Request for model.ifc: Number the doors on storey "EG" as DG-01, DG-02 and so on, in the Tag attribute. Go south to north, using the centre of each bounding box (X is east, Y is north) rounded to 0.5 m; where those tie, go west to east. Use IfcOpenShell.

First a look at what the model holds.

```python
import ifcopenshell
import ifcopenshell.util.element
import ifcopenshell.util.placement

model = ifcopenshell.open("model.ifc")
print(model.schema)
storey = next(s for s in model.by_type("IfcBuildingStorey") if s.Name == "EG")
doors = [e for e in ifcopenshell.util.element.get_decomposition(storey) if e.is_a("IfcDoor")]
for e in sorted(doors, key=lambda e: e.id()):
    origin = ifcopenshell.util.placement.get_local_placement(e.ObjectPlacement)[:3, 3]
    print(e.id(), e.Tag, e.Name, origin.round(2) + 0.0, sep=" | ")
```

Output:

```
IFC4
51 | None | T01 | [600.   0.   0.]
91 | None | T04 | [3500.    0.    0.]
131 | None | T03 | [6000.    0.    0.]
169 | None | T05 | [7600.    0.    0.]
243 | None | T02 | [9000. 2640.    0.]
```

```python
import ifcopenshell
import ifcopenshell.geom
import ifcopenshell.util.element
import ifcopenshell.util.shape

model = ifcopenshell.open("model.ifc")
settings = ifcopenshell.geom.settings()
settings.set("use-world-coords", True)


def centre(element):
    shape = ifcopenshell.geom.create_shape(settings, element)
    return ifcopenshell.util.shape.get_bbox_centroid(shape.geometry)


storey = next(s for s in model.by_type("IfcBuildingStorey") if s.Name == "EG")
doors = [e for e in ifcopenshell.util.element.get_decomposition(storey) if e.is_a("IfcDoor")]

# Insertion points can sit at a corner or the storey origin, so sort by the geometry (in metres).
centres = {e: centre(e) for e in doors}
doors.sort(key=lambda e: (round(centres[e][1] / 0.5), centres[e][0]))

for i, e in enumerate(doors, start=1):
    number = f"DG-{i:02d}"
    e.Tag = number
    print(e.id(), number)

model.write("model_rev.ifc")
```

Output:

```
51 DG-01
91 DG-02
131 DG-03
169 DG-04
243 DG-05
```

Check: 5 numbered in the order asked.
